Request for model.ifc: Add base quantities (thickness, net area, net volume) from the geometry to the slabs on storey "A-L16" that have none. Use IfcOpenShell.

First a look at what the model holds.

```python
import ifcopenshell
import ifcopenshell.util.element
import ifcopenshell.util.unit

model = ifcopenshell.open("model.ifc")
print(model.schema)
for unit_type in ("LENGTHUNIT", "AREAUNIT", "VOLUMEUNIT"):
    print(unit_type, ifcopenshell.util.unit.calculate_unit_scale(model, unit_type))
storey = next(s for s in model.by_type("IfcBuildingStorey") if s.Name == "A-L16")
slabs = [e for e in ifcopenshell.util.element.get_decomposition(storey) if e.is_a("IfcSlab")]
for e in sorted(slabs, key=lambda e: e.id()):
    print(e.id(), e.is_a(), e.Name, list(ifcopenshell.util.element.get_psets(e, qtos_only=True)), sep=" | ")
```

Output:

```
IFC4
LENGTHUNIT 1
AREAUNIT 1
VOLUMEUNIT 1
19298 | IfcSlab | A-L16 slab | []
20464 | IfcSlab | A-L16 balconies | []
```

```python
import ifcopenshell
import ifcopenshell.api.pset
import ifcopenshell.geom
import ifcopenshell.util.element
import ifcopenshell.util.shape
import ifcopenshell.util.unit

model = ifcopenshell.open("model.ifc")
unit_scale = ifcopenshell.util.unit.calculate_unit_scale(model)
area_scale = ifcopenshell.util.unit.calculate_unit_scale(model, "AREAUNIT")
volume_scale = ifcopenshell.util.unit.calculate_unit_scale(model, "VOLUMEUNIT")
settings = ifcopenshell.geom.settings()

storey = next(s for s in model.by_type("IfcBuildingStorey") if s.Name == "A-L16")
slabs = [e for e in ifcopenshell.util.element.get_decomposition(storey) if e.is_a("IfcSlab")]

for e in sorted(slabs, key=lambda e: e.id()):
    if ifcopenshell.util.element.get_psets(e, qtos_only=True, should_inherit=False):
        continue
    # Geometry comes back in metres, in the element's own axes.
    shape = ifcopenshell.geom.create_shape(settings, e)
    values = {
        "Width": ifcopenshell.util.shape.get_z(shape.geometry) / unit_scale,
        "NetArea": ifcopenshell.util.shape.get_footprint_area(shape.geometry) / area_scale,
        "NetVolume": ifcopenshell.util.shape.get_volume(shape.geometry) / volume_scale,
    }
    qto = ifcopenshell.api.pset.add_qto(model, product=e, name="Qto_SlabBaseQuantities")
    ifcopenshell.api.pset.edit_qto(model, qto=qto, properties=values)
    print(e.id(), {k: round(v, 3) for k, v in values.items()})

model.write("model_updated.ifc")
```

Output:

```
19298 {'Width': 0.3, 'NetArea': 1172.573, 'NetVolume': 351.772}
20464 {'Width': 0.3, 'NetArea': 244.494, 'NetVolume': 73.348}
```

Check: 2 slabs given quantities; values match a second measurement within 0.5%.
